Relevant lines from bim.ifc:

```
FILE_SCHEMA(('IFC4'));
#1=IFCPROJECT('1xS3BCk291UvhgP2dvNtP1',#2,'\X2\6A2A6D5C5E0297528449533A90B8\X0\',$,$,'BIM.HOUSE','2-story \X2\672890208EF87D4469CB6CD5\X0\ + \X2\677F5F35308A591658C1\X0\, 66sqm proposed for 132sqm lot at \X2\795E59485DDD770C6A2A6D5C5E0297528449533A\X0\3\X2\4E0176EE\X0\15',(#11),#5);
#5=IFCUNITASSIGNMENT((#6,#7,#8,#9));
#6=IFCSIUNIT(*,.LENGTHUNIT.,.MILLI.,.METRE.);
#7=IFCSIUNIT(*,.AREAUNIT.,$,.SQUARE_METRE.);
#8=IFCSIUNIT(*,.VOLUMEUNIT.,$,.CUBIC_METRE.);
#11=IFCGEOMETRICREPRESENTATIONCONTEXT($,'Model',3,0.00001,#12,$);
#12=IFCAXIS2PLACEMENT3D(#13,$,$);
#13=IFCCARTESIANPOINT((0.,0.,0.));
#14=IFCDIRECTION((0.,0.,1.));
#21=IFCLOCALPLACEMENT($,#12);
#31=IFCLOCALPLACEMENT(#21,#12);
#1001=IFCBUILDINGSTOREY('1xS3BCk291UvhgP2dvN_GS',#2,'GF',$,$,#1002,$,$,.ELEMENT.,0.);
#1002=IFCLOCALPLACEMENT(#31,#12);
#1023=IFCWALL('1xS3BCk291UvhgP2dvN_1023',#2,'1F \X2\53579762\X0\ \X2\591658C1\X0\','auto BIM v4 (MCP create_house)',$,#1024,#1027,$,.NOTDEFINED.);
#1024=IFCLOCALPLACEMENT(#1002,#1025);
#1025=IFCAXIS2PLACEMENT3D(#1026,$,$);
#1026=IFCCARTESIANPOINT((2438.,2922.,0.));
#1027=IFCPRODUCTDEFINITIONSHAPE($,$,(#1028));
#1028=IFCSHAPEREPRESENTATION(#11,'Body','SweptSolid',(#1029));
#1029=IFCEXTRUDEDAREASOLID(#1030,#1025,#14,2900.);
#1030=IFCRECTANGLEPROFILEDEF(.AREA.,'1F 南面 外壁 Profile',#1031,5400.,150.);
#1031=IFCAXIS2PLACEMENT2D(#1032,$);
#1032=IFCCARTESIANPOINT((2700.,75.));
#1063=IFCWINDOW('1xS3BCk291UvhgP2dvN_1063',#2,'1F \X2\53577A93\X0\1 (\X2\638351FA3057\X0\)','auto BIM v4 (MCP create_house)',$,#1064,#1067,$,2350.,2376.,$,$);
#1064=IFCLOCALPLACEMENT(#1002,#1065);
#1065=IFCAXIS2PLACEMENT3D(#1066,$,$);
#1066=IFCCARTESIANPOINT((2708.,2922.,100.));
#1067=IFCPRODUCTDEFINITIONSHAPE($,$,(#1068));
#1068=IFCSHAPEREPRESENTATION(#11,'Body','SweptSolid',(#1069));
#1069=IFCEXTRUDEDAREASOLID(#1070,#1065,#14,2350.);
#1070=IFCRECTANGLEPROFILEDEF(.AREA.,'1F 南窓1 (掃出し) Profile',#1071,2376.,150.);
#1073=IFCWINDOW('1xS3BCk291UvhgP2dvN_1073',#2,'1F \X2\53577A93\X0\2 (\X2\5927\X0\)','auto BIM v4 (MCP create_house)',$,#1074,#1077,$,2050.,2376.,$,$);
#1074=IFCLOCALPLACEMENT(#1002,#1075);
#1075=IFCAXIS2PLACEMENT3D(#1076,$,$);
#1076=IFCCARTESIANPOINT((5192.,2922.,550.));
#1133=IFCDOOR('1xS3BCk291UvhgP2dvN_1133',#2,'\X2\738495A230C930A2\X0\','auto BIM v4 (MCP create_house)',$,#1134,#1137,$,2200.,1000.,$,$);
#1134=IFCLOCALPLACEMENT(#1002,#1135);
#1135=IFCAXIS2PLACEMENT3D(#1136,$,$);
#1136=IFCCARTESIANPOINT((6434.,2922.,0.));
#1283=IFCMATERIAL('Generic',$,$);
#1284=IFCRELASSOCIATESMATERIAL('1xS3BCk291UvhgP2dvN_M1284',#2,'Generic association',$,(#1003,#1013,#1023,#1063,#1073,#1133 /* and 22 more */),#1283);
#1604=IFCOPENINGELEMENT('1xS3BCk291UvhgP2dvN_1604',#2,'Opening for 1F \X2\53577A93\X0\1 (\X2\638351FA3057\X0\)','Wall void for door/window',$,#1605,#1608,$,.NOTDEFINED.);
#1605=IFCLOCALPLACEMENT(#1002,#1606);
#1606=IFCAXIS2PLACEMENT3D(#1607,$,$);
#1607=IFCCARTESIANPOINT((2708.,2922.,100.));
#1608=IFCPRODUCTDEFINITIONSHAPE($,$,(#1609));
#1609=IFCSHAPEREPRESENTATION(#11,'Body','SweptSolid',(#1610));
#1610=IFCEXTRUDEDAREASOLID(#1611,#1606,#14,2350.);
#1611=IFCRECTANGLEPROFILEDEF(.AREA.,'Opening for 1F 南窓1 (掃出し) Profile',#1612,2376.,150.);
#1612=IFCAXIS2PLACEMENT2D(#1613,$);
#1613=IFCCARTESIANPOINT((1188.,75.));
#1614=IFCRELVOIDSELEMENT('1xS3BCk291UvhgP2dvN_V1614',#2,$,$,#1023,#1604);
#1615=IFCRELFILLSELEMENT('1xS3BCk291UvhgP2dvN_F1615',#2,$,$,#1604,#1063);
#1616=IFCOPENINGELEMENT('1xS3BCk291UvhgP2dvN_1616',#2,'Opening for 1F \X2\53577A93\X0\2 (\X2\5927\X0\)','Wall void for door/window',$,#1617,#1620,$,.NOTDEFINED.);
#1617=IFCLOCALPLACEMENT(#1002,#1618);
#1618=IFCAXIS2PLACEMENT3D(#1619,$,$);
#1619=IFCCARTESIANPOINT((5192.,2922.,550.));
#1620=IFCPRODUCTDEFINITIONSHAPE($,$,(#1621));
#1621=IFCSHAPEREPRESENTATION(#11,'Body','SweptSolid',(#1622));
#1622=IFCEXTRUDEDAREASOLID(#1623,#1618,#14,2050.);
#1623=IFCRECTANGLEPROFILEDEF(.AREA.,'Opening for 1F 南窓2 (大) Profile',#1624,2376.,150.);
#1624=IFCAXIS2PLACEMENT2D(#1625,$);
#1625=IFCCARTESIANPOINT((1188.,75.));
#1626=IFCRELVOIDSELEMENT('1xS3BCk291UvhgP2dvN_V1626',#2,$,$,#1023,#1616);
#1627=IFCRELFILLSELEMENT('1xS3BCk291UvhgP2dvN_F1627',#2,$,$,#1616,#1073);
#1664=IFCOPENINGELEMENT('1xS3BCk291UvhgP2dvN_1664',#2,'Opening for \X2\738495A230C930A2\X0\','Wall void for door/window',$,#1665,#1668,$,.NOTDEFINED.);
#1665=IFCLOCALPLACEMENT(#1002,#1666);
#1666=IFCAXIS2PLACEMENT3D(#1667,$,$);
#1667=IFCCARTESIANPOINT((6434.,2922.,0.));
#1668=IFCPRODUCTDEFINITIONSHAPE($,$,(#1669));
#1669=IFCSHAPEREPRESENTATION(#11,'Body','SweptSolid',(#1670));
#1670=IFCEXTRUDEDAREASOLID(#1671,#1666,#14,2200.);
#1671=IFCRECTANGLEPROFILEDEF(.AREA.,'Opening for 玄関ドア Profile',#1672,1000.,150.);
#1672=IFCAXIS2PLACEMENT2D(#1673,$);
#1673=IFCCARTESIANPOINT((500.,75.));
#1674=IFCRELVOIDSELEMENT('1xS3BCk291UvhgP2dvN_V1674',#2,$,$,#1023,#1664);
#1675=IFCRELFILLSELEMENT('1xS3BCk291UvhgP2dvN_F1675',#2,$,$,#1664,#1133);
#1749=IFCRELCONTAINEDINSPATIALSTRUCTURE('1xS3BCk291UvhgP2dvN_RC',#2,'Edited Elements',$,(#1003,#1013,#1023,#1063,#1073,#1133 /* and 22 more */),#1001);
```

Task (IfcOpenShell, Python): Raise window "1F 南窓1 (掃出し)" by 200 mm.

```python
import numpy as np
import ifcopenshell
import ifcopenshell.api.geometry
import ifcopenshell.util.placement
import ifcopenshell.util.unit

model = ifcopenshell.open("bim.ifc")
unit_scale = ifcopenshell.util.unit.calculate_unit_scale(model)

window = model.by_id(1063)
opening = window.FillsVoids[0].RelatingOpeningElement
dz = 0.2 / unit_scale

shift = np.array([0.0, 0.0, dz])
# The window is not placed relative to its opening, so move both.
for product in (opening, window):
    matrix = ifcopenshell.util.placement.get_local_placement(product.ObjectPlacement)
    matrix[:3, 3] += shift
    ifcopenshell.api.geometry.edit_object_placement(model, product=product, matrix=matrix, is_si=False)

print(f"moved by {dz * unit_scale:+.3f} m")

model.write("bim_v2.ifc")
```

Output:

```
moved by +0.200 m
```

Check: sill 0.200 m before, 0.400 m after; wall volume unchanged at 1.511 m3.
